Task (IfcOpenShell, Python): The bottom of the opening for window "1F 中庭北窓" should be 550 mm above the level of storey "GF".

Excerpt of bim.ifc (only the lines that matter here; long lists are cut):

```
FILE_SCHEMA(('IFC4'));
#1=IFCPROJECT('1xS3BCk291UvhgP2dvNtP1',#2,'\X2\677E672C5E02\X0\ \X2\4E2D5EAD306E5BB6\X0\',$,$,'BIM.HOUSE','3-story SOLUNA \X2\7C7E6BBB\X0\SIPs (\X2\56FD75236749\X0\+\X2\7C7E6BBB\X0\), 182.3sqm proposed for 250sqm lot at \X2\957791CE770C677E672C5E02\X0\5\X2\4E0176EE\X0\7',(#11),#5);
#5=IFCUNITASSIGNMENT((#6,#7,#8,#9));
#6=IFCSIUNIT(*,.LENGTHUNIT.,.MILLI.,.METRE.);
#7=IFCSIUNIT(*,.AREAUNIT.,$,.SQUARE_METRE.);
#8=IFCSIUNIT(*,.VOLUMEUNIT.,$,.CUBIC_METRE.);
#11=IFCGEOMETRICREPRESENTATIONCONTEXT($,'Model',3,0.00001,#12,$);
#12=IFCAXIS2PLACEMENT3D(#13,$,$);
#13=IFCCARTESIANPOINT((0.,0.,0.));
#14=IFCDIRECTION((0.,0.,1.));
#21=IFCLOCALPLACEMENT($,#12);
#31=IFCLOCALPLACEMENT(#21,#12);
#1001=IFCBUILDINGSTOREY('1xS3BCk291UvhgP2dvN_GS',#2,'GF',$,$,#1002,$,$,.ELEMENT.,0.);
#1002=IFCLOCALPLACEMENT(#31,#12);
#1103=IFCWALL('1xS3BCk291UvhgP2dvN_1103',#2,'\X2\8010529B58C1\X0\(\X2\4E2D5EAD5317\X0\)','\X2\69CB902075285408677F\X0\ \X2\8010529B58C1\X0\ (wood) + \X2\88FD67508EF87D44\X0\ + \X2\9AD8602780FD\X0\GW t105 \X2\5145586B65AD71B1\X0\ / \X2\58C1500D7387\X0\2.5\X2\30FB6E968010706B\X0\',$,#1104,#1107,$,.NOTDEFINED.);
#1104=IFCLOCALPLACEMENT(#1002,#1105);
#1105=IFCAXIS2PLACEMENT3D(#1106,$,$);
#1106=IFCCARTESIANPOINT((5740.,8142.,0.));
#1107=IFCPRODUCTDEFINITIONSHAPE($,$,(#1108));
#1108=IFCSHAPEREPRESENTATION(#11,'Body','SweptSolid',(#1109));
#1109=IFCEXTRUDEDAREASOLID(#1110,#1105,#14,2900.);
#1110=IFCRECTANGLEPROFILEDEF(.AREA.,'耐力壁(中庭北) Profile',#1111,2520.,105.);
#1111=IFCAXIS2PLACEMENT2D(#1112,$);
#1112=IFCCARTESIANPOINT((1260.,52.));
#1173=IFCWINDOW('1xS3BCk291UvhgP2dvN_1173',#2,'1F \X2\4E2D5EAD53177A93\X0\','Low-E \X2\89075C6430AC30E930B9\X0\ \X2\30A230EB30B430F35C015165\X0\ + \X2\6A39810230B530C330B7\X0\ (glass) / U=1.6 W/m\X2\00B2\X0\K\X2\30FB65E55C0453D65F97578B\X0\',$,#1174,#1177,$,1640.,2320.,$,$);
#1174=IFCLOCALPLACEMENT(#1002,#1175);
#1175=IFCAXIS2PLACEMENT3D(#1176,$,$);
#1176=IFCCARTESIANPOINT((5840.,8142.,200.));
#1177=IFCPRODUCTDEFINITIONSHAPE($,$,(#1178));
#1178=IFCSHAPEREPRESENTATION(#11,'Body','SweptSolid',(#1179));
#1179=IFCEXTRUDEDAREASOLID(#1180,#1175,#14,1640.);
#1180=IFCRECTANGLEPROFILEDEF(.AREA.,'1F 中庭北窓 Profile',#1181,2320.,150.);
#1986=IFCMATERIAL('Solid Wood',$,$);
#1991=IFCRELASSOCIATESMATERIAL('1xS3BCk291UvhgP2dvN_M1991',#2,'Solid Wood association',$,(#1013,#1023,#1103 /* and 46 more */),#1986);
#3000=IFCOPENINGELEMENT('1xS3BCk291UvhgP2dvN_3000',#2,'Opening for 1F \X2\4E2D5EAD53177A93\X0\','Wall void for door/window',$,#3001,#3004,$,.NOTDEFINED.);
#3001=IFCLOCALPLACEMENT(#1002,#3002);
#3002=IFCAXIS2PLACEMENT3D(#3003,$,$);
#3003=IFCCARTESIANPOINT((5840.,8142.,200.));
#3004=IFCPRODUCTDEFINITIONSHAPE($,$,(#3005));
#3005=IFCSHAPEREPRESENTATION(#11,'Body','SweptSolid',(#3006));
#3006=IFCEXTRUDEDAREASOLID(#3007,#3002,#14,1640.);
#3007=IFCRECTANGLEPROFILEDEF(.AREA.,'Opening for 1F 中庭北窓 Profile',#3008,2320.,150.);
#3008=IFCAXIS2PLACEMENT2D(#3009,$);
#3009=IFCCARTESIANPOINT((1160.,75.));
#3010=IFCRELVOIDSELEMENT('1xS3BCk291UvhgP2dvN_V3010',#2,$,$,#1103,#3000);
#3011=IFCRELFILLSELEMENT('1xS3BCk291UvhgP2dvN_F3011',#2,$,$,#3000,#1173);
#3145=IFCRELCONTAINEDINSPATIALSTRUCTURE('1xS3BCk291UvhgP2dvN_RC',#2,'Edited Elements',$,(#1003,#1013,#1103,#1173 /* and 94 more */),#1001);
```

```python
import numpy as np
import ifcopenshell
import ifcopenshell.api.geometry
import ifcopenshell.geom
import ifcopenshell.util.element
import ifcopenshell.util.placement
import ifcopenshell.util.shape
import ifcopenshell.util.unit

model = ifcopenshell.open("bim.ifc")
unit_scale = ifcopenshell.util.unit.calculate_unit_scale(model)

window = model.by_id(1173)
opening = window.FillsVoids[0].RelatingOpeningElement
storey = ifcopenshell.util.element.get_container(window, ifc_class="IfcBuildingStorey")
level = ifcopenshell.util.placement.get_local_placement(storey.ObjectPlacement)[2, 3]

# The opening's origin need not be at the sill, so measure its lowest point.
shape = ifcopenshell.geom.create_shape(ifcopenshell.geom.settings(), opening)
bottom = ifcopenshell.util.shape.get_shape_bottom_elevation(shape, shape.geometry) / unit_scale
dz = level + 550.0 - bottom

shift = np.array([0.0, 0.0, dz])
# The window is not placed relative to its opening, so move both.
for product in (opening, window):
    matrix = ifcopenshell.util.placement.get_local_placement(product.ObjectPlacement)
    matrix[:3, 3] += shift
    ifcopenshell.api.geometry.edit_object_placement(model, product=product, matrix=matrix, is_si=False)

print(f"moved by {dz * unit_scale:+.3f} m")

model.write("bim_edited.ifc")
```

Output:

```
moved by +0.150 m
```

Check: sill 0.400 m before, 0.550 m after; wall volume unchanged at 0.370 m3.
